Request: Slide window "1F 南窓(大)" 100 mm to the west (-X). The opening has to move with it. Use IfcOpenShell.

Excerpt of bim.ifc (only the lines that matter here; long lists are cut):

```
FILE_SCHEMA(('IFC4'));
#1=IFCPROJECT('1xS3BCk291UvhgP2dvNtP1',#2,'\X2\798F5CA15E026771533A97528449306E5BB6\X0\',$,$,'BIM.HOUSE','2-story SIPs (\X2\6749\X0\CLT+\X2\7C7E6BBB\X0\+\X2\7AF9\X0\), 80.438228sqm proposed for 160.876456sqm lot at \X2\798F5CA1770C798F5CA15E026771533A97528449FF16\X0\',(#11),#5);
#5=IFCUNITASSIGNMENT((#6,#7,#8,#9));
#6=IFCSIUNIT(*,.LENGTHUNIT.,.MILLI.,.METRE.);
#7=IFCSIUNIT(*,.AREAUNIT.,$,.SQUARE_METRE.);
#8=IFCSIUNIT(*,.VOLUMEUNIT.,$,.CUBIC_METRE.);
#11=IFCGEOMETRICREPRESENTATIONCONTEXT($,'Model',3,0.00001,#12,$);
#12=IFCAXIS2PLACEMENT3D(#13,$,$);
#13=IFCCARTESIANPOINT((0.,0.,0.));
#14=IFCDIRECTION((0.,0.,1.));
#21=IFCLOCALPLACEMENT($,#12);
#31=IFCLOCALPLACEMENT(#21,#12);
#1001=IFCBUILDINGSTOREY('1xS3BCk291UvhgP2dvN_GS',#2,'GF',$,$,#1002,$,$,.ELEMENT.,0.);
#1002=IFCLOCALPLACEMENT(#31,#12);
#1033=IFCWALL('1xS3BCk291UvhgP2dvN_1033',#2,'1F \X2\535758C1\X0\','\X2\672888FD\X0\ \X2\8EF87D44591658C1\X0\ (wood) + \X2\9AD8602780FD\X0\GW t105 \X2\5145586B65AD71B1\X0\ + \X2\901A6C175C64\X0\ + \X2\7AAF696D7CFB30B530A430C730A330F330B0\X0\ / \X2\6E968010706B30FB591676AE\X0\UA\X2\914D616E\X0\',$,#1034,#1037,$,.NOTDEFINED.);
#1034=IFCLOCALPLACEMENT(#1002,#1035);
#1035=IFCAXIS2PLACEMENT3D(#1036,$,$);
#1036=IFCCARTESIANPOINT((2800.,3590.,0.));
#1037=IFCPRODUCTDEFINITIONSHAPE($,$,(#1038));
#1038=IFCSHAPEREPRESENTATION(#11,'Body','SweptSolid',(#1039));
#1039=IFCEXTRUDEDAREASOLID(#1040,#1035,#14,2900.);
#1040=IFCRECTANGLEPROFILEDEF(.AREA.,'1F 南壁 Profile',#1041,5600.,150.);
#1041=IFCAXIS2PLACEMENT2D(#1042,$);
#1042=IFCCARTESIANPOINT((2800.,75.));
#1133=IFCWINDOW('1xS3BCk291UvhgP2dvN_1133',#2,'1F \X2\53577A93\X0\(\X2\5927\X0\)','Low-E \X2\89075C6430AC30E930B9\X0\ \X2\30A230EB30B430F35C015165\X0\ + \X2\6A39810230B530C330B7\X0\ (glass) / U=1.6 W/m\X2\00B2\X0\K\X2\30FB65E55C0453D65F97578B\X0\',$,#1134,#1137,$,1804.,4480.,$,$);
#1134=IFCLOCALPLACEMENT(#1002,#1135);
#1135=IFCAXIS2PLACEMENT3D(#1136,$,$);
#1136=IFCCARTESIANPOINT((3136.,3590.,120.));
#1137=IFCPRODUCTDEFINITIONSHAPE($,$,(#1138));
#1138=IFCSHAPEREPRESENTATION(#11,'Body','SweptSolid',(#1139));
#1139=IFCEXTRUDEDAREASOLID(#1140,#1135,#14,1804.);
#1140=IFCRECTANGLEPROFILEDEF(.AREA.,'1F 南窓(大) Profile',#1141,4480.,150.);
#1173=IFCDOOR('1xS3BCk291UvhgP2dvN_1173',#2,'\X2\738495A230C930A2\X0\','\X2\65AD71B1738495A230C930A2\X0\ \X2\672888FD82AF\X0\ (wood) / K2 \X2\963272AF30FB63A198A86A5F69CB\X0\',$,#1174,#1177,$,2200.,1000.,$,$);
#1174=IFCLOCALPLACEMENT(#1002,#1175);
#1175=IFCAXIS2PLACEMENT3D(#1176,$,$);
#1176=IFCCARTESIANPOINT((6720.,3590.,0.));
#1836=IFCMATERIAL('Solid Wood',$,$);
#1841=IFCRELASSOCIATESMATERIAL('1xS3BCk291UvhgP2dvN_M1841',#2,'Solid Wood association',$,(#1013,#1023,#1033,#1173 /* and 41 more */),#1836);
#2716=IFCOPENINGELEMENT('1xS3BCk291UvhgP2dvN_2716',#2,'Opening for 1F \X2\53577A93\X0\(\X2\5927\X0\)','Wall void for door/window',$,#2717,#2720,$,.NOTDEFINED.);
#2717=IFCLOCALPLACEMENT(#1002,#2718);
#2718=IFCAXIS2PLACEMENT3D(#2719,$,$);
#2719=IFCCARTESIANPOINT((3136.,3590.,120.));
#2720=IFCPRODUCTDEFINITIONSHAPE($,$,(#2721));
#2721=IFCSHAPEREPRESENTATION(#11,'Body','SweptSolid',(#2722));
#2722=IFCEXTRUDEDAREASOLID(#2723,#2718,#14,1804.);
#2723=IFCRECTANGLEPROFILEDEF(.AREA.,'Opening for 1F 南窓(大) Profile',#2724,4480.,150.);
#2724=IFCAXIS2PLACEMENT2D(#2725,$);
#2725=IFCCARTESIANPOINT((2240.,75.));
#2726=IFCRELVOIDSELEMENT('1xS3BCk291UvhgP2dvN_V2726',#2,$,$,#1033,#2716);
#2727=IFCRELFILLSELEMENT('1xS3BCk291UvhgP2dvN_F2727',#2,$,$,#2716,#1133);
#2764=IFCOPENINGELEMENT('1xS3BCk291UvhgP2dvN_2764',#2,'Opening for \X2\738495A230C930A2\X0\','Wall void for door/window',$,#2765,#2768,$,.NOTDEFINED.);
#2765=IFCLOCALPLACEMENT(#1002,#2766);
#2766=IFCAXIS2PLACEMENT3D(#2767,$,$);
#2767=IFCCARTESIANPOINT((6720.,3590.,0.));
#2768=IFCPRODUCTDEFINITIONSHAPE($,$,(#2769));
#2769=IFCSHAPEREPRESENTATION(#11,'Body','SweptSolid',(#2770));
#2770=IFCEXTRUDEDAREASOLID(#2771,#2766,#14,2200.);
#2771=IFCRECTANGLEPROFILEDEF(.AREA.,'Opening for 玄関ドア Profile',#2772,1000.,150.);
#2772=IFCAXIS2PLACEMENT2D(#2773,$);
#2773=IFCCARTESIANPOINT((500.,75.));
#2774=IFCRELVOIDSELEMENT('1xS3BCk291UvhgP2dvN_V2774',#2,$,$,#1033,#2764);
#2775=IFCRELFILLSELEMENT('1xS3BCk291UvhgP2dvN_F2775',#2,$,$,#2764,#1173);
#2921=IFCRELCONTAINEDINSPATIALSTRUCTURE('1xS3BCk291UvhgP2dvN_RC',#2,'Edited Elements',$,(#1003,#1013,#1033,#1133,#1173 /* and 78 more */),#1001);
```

```python
import ifcopenshell
import ifcopenshell.api.geometry
import ifcopenshell.util.placement
import ifcopenshell.util.unit

model = ifcopenshell.open("bim.ifc")
unit_scale = ifcopenshell.util.unit.calculate_unit_scale(model)

window = model.by_guid("1xS3BCk291UvhgP2dvN_1133")
opening = window.FillsVoids[0].RelatingOpeningElement
wall = opening.VoidsElements[0].RelatingBuildingElement

wall_matrix = ifcopenshell.util.placement.get_local_placement(wall.ObjectPlacement)
shift = wall_matrix[:3, 0] * -0.1 / unit_scale
before = ifcopenshell.util.placement.get_local_placement(window.ObjectPlacement)[:3, 3].copy()

# The window is not placed relative to its opening, so move both.
for product in (opening, window):
    matrix = ifcopenshell.util.placement.get_local_placement(product.ObjectPlacement)
    matrix[:3, 3] += shift
    ifcopenshell.api.geometry.edit_object_placement(model, product=product, matrix=matrix, is_si=False)

after = ifcopenshell.util.placement.get_local_placement(window.ObjectPlacement)[:3, 3]
print("window moved by", (after - before).round(3) + 0.0)

model.write("bim_updated.ifc")
```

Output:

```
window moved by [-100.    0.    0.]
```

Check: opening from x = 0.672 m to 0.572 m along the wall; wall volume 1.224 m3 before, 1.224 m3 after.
